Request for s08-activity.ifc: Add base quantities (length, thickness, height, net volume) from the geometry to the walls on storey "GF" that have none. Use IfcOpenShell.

First a look at what the model holds.

```python
import ifcopenshell
import ifcopenshell.util.element
import ifcopenshell.util.unit

model = ifcopenshell.open("s08-activity.ifc")
print(model.schema)
for unit_type in ("LENGTHUNIT", "AREAUNIT", "VOLUMEUNIT"):
    print(unit_type, ifcopenshell.util.unit.calculate_unit_scale(model, unit_type))
storey = next(s for s in model.by_type("IfcBuildingStorey") if s.Name == "GF")
walls = [e for e in ifcopenshell.util.element.get_decomposition(storey) if e.is_a("IfcWall")]
for e in sorted(walls, key=lambda e: e.id()):
    print(e.id(), e.is_a(), e.Name, list(ifcopenshell.util.element.get_psets(e, qtos_only=True)), sep=" | ")
```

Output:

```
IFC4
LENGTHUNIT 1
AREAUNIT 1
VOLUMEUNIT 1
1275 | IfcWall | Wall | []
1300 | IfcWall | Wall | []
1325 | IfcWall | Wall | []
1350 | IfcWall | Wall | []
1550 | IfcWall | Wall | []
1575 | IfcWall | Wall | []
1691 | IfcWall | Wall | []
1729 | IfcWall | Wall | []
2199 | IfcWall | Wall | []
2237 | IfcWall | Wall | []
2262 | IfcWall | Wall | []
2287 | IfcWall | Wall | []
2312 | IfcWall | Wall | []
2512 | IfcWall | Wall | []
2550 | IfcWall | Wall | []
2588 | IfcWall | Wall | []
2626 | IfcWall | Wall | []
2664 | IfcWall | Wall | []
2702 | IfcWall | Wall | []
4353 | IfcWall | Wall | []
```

```python
import ifcopenshell
import ifcopenshell.api.pset
import ifcopenshell.geom
import ifcopenshell.util.element
import ifcopenshell.util.shape
import ifcopenshell.util.unit

model = ifcopenshell.open("s08-activity.ifc")
unit_scale = ifcopenshell.util.unit.calculate_unit_scale(model)
volume_scale = ifcopenshell.util.unit.calculate_unit_scale(model, "VOLUMEUNIT")
settings = ifcopenshell.geom.settings()

storey = next(s for s in model.by_type("IfcBuildingStorey") if s.Name == "GF")
walls = [e for e in ifcopenshell.util.element.get_decomposition(storey) if e.is_a("IfcWall")]

for e in sorted(walls, key=lambda e: e.id()):
    if ifcopenshell.util.element.get_psets(e, qtos_only=True, should_inherit=False):
        continue
    # Geometry comes back in metres, in the element's own axes.
    shape = ifcopenshell.geom.create_shape(settings, e)
    values = {
        "Length": ifcopenshell.util.shape.get_x(shape.geometry) / unit_scale,
        "Width": ifcopenshell.util.shape.get_y(shape.geometry) / unit_scale,
        "Height": ifcopenshell.util.shape.get_z(shape.geometry) / unit_scale,
        "NetVolume": ifcopenshell.util.shape.get_volume(shape.geometry) / volume_scale,
    }
    qto = ifcopenshell.api.pset.add_qto(model, product=e, name="Qto_WallBaseQuantities")
    ifcopenshell.api.pset.edit_qto(model, qto=qto, properties=values)
    print(e.id(), {k: round(v, 3) for k, v in values.items()})

model.write("s08-activity_v2.ifc")
```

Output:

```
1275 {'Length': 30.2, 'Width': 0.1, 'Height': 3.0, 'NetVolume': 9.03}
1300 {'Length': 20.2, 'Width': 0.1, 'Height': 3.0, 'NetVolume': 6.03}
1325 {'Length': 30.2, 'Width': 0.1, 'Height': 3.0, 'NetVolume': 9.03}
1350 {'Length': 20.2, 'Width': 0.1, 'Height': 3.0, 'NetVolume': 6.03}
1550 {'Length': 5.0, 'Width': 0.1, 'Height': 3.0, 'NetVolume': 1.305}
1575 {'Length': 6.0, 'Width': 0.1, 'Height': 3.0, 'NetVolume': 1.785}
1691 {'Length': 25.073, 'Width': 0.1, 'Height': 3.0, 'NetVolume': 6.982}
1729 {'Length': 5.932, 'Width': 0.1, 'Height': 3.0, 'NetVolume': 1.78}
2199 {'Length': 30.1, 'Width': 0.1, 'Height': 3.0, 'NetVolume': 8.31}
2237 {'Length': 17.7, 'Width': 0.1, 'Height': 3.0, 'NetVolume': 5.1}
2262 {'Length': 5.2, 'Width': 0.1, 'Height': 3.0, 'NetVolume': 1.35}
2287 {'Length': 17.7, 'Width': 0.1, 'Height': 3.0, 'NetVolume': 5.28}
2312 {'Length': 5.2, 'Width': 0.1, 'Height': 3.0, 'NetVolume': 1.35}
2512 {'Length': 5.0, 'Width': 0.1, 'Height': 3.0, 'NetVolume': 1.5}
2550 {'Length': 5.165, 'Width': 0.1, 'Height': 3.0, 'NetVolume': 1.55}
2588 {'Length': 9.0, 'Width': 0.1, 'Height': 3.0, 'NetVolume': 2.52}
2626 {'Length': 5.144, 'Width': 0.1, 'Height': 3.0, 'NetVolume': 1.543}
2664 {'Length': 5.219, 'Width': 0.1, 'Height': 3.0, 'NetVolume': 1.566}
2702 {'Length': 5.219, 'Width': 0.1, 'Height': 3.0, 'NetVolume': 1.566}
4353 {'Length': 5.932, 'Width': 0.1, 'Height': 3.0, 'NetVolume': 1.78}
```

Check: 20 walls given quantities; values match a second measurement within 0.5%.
